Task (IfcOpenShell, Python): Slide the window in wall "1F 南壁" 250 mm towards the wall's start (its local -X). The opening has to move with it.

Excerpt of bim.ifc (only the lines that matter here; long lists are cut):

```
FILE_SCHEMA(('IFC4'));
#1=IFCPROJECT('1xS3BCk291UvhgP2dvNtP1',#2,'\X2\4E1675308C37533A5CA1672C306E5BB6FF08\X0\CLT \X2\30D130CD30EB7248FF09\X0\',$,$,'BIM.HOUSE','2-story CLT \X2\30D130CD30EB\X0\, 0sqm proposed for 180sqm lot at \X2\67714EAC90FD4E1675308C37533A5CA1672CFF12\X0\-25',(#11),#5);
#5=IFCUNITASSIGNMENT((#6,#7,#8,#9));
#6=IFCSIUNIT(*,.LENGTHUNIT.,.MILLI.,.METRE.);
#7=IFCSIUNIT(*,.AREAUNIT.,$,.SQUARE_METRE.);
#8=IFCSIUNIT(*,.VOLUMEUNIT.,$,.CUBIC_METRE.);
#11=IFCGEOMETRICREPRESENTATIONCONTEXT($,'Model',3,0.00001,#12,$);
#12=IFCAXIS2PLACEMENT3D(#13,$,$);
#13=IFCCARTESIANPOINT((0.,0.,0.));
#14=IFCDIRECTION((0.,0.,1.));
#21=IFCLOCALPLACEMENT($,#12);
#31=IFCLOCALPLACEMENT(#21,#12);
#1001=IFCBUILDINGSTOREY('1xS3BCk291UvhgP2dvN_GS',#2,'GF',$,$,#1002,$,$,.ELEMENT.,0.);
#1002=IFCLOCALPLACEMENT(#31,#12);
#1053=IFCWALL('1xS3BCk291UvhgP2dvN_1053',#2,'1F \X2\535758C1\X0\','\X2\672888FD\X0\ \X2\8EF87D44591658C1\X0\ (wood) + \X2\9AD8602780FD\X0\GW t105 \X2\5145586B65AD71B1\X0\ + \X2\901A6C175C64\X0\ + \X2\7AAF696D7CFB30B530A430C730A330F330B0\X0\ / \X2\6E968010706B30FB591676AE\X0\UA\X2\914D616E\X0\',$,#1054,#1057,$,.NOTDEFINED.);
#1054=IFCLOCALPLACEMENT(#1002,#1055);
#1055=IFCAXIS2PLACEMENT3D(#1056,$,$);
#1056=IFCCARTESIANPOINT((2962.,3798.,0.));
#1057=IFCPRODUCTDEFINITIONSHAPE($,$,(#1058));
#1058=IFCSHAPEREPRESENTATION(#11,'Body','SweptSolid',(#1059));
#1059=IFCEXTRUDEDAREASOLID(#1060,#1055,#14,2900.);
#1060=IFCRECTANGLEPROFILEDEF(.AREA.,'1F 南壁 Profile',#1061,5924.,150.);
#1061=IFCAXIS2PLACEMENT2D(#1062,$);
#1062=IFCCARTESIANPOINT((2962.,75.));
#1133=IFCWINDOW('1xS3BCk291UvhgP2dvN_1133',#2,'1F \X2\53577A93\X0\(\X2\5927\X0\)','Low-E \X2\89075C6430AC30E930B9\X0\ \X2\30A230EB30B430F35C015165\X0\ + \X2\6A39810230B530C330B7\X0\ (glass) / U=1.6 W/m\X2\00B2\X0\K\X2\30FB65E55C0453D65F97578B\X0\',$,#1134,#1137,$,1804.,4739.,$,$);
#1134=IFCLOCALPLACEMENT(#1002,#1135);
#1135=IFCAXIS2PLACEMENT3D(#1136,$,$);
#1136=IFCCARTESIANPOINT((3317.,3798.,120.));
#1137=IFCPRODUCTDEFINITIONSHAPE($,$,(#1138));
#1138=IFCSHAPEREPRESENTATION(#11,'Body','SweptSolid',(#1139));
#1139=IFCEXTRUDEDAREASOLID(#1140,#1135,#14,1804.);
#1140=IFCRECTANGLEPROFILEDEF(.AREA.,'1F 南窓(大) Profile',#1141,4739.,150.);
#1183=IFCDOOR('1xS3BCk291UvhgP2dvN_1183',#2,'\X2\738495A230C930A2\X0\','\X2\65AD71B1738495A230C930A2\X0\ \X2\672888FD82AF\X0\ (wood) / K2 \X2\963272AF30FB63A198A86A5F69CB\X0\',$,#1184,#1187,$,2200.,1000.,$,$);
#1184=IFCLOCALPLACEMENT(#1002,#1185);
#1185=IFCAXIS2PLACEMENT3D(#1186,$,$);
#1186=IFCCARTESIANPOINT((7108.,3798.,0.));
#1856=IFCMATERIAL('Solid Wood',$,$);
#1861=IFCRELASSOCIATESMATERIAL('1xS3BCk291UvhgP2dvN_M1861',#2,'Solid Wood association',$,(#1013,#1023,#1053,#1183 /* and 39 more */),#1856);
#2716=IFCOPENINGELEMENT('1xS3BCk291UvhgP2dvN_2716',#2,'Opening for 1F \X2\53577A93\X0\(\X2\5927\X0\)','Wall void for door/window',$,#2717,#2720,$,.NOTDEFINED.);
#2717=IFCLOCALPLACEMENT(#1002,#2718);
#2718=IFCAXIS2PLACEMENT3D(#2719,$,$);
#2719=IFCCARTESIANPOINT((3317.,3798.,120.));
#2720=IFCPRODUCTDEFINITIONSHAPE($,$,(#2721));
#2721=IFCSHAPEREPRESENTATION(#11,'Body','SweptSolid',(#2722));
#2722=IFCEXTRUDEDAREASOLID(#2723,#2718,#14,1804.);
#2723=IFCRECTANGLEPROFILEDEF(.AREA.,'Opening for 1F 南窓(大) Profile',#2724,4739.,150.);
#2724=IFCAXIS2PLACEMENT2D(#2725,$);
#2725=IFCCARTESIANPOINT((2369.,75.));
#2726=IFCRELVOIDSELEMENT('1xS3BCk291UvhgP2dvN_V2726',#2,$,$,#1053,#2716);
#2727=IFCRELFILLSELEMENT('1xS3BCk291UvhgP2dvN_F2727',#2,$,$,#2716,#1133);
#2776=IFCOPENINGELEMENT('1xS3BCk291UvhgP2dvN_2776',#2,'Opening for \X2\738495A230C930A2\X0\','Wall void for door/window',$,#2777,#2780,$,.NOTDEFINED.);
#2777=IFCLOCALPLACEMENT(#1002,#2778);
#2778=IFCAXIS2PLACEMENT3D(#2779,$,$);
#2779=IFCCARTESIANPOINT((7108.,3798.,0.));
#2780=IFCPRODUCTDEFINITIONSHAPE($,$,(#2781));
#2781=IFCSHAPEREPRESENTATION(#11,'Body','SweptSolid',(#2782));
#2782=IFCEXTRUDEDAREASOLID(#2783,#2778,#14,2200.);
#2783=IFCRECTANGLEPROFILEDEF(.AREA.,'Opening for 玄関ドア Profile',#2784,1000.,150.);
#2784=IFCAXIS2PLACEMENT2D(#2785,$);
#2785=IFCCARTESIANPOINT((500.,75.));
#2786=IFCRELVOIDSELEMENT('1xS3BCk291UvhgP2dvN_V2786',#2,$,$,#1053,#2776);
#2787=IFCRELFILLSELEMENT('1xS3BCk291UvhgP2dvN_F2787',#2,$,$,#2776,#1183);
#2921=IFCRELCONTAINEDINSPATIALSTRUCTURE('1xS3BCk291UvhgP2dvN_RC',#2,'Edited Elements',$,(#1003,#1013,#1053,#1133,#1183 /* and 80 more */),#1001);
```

```python
import ifcopenshell
import ifcopenshell.api.geometry
import ifcopenshell.util.placement

model = ifcopenshell.open("bim.ifc")

window = model.by_id(1133)
opening = window.FillsVoids[0].RelatingOpeningElement
wall = opening.VoidsElements[0].RelatingBuildingElement

wall_matrix = ifcopenshell.util.placement.get_local_placement(wall.ObjectPlacement)
shift = wall_matrix[:3, 0] * -250.0
before = ifcopenshell.util.placement.get_local_placement(window.ObjectPlacement)[:3, 3].copy()

# The window is not placed relative to its opening, so move both.
for product in (opening, window):
    matrix = ifcopenshell.util.placement.get_local_placement(product.ObjectPlacement)
    matrix[:3, 3] += shift
    ifcopenshell.api.geometry.edit_object_placement(model, product=product, matrix=matrix, is_si=False)

after = ifcopenshell.util.placement.get_local_placement(window.ObjectPlacement)[:3, 3]
print("window moved by", (after - before).round(3) + 0.0)

model.write("bim_rev.ifc")
```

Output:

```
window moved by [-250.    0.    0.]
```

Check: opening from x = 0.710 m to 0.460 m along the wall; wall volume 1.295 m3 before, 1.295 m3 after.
